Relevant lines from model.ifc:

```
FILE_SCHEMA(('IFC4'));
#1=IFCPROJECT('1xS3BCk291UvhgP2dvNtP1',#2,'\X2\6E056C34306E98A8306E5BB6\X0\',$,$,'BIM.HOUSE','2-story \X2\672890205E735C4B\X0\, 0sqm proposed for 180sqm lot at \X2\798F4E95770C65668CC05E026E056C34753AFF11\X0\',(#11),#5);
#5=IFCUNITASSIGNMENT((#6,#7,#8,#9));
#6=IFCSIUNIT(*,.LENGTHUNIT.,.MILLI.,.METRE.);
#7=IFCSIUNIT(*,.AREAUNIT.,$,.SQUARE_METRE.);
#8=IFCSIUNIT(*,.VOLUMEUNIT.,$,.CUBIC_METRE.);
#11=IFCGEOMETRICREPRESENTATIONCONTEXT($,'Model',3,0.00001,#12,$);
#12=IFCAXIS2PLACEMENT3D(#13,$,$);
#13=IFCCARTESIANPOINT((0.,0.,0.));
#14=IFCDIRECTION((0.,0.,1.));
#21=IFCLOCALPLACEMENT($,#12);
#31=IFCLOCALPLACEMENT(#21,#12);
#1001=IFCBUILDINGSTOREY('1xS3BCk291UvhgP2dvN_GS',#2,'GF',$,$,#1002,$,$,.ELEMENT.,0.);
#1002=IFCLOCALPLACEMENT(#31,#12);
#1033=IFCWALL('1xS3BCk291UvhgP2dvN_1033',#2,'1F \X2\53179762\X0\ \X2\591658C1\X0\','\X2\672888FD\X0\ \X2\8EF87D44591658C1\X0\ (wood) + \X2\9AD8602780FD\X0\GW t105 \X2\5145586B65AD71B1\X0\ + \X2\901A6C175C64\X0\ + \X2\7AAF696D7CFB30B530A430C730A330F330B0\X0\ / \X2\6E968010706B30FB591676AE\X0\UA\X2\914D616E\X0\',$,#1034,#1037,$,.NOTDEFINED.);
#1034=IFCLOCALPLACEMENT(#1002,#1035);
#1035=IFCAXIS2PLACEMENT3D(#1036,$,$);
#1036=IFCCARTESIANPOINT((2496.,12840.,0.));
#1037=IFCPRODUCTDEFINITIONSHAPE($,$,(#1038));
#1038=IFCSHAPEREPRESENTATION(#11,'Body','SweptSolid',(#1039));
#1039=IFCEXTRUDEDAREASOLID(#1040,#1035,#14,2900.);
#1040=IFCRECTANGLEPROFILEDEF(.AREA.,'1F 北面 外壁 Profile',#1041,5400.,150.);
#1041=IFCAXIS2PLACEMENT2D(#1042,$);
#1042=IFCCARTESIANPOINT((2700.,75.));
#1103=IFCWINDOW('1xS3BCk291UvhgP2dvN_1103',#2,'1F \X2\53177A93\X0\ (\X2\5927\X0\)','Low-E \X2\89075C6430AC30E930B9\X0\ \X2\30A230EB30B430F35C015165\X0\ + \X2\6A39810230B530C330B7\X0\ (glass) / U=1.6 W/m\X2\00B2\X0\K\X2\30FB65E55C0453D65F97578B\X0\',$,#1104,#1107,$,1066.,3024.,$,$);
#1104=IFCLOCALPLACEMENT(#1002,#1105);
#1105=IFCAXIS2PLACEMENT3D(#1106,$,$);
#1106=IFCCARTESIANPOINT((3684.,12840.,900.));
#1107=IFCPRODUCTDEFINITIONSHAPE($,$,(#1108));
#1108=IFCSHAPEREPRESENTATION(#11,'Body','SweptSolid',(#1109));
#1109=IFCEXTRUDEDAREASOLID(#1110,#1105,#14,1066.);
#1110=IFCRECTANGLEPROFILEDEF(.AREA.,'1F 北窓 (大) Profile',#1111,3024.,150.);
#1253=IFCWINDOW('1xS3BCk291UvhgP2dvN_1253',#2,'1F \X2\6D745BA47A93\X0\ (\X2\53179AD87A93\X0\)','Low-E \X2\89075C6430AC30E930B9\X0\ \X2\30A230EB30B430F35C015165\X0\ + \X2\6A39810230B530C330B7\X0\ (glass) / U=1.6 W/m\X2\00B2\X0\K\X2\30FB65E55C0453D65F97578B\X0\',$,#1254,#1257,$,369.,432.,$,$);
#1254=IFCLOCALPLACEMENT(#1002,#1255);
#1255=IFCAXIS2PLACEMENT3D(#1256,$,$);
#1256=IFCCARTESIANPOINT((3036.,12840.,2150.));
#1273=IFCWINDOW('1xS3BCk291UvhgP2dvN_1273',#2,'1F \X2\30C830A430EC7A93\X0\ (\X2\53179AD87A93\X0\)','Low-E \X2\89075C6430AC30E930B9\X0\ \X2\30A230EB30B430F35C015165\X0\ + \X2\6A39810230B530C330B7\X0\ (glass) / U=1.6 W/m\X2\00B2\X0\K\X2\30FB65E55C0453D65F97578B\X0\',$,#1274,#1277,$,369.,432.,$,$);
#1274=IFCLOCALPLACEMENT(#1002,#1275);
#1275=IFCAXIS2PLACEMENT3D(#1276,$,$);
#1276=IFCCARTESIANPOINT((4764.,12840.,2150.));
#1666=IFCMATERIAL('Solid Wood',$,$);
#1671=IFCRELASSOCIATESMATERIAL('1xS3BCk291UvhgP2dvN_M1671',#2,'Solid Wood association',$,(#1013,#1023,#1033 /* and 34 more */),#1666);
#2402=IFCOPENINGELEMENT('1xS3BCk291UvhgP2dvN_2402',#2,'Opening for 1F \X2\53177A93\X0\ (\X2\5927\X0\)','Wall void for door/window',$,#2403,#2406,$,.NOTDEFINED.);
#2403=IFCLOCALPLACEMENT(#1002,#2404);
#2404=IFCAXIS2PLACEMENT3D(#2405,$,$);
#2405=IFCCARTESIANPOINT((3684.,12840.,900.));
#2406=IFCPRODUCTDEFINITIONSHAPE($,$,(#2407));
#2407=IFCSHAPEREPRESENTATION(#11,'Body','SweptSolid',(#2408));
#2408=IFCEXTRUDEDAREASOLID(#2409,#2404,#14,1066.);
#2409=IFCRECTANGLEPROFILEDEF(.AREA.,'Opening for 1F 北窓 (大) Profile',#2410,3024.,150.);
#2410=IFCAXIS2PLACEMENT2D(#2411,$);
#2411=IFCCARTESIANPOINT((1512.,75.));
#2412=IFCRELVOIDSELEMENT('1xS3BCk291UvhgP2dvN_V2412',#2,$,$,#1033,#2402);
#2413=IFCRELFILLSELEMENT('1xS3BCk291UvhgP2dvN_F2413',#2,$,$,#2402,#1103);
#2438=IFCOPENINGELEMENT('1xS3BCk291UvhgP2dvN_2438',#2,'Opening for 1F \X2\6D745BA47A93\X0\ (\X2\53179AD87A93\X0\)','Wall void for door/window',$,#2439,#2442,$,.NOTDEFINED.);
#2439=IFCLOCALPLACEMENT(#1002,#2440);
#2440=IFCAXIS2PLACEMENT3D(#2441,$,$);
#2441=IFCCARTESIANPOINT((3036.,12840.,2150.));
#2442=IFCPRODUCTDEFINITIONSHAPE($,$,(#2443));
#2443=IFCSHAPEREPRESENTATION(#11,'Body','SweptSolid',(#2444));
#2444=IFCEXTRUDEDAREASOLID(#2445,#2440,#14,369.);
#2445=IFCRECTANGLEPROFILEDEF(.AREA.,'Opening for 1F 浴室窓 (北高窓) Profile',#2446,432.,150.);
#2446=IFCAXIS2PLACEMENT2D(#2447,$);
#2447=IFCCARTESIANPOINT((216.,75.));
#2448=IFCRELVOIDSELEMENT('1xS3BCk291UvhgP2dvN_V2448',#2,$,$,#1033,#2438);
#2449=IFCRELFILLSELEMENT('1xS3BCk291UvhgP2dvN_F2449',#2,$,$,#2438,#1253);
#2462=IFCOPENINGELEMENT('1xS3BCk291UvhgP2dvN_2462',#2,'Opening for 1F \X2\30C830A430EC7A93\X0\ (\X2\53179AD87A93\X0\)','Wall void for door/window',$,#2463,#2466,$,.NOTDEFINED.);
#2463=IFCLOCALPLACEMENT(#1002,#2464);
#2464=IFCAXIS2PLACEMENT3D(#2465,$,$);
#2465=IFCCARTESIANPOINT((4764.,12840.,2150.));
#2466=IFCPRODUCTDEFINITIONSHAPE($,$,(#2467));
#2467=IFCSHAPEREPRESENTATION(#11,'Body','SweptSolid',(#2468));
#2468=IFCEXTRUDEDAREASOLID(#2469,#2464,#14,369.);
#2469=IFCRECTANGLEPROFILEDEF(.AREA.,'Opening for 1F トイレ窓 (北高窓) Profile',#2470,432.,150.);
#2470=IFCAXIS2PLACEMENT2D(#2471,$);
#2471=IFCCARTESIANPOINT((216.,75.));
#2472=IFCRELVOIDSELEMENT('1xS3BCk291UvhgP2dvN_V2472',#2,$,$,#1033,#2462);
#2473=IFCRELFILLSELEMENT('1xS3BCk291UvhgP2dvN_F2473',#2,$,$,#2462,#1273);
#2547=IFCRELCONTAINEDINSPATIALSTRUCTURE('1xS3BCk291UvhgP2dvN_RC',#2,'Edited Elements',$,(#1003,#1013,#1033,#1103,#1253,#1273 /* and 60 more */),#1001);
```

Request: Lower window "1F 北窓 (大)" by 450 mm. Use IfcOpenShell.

```python
import numpy as np
import ifcopenshell
import ifcopenshell.api.geometry
import ifcopenshell.util.placement
import ifcopenshell.util.unit

model = ifcopenshell.open("model.ifc")
unit_scale = ifcopenshell.util.unit.calculate_unit_scale(model)

window = model.by_guid("1xS3BCk291UvhgP2dvN_1103")
opening = window.FillsVoids[0].RelatingOpeningElement
dz = -0.45 / unit_scale

shift = np.array([0.0, 0.0, dz])
# The window is not placed relative to its opening, so move both.
for product in (opening, window):
    matrix = ifcopenshell.util.placement.get_local_placement(product.ObjectPlacement)
    matrix[:3, 3] += shift
    ifcopenshell.api.geometry.edit_object_placement(model, product=product, matrix=matrix, is_si=False)

print(f"moved by {dz * unit_scale:+.3f} m")

model.write("model_edited.ifc")
```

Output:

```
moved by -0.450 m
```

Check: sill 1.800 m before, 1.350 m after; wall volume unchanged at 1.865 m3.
